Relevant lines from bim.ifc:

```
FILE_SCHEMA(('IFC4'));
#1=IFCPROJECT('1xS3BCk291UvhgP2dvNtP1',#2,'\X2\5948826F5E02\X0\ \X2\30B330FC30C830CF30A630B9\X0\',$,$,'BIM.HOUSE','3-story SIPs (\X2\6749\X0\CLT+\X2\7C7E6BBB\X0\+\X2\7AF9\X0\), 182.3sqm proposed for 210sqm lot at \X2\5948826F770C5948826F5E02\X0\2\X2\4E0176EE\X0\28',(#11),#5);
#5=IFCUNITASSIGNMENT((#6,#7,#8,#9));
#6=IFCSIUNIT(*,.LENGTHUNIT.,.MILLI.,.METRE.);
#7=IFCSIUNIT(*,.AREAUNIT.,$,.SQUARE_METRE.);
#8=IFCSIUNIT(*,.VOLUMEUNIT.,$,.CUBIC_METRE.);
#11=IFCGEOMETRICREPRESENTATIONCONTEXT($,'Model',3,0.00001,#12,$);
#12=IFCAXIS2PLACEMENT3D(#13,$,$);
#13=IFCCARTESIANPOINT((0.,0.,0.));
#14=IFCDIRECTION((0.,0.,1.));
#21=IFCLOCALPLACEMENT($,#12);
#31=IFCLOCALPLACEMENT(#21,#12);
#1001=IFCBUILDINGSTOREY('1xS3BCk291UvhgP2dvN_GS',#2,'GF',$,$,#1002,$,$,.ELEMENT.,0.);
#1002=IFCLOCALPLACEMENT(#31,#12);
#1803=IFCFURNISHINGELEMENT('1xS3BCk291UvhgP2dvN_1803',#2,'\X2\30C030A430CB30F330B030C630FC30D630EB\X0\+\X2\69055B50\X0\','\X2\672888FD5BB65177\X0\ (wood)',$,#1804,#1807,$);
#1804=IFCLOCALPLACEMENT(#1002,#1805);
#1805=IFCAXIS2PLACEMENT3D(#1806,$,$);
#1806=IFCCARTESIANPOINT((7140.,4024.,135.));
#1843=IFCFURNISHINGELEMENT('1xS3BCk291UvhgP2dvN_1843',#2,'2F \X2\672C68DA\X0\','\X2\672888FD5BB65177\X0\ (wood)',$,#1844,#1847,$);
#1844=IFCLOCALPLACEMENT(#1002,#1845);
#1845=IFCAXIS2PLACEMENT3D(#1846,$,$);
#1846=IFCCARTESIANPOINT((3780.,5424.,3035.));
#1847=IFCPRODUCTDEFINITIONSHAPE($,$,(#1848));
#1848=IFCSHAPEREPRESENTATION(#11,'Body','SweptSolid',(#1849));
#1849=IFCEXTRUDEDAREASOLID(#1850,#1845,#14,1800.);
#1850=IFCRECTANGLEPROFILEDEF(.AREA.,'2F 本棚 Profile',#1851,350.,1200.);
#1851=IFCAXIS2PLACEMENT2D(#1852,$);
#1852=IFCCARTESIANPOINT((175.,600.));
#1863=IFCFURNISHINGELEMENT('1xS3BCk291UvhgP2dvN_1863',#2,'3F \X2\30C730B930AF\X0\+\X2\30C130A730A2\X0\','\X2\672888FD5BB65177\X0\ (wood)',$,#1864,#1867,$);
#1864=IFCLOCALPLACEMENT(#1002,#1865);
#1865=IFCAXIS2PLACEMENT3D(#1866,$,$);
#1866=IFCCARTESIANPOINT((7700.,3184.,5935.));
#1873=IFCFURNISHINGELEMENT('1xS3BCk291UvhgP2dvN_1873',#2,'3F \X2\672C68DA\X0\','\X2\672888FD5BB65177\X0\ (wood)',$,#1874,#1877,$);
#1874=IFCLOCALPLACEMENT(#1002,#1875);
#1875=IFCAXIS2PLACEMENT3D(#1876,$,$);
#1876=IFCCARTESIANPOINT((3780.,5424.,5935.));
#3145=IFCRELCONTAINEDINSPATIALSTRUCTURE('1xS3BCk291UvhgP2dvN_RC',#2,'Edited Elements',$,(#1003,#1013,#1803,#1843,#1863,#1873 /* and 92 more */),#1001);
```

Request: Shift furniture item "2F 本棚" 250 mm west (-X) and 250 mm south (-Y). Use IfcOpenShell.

```python
import ifcopenshell
import ifcopenshell.api.geometry
import ifcopenshell.util.placement
import ifcopenshell.util.unit

model = ifcopenshell.open("bim.ifc")
unit_scale = ifcopenshell.util.unit.calculate_unit_scale(model)

item = model.by_guid("1xS3BCk291UvhgP2dvN_1843")
matrix = ifcopenshell.util.placement.get_local_placement(item.ObjectPlacement)
matrix[0, 3] -= 0.25 / unit_scale
matrix[1, 3] -= 0.25 / unit_scale
ifcopenshell.api.geometry.edit_object_placement(model, product=item, matrix=matrix, is_si=False)

print(ifcopenshell.util.placement.get_local_placement(item.ObjectPlacement).round(3) + 0.0)

model.write("bim_edited.ifc")
```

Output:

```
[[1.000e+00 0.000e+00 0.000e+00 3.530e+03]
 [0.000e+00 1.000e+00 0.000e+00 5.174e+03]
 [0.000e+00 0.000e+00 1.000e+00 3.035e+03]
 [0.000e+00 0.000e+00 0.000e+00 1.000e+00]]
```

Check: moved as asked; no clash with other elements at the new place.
